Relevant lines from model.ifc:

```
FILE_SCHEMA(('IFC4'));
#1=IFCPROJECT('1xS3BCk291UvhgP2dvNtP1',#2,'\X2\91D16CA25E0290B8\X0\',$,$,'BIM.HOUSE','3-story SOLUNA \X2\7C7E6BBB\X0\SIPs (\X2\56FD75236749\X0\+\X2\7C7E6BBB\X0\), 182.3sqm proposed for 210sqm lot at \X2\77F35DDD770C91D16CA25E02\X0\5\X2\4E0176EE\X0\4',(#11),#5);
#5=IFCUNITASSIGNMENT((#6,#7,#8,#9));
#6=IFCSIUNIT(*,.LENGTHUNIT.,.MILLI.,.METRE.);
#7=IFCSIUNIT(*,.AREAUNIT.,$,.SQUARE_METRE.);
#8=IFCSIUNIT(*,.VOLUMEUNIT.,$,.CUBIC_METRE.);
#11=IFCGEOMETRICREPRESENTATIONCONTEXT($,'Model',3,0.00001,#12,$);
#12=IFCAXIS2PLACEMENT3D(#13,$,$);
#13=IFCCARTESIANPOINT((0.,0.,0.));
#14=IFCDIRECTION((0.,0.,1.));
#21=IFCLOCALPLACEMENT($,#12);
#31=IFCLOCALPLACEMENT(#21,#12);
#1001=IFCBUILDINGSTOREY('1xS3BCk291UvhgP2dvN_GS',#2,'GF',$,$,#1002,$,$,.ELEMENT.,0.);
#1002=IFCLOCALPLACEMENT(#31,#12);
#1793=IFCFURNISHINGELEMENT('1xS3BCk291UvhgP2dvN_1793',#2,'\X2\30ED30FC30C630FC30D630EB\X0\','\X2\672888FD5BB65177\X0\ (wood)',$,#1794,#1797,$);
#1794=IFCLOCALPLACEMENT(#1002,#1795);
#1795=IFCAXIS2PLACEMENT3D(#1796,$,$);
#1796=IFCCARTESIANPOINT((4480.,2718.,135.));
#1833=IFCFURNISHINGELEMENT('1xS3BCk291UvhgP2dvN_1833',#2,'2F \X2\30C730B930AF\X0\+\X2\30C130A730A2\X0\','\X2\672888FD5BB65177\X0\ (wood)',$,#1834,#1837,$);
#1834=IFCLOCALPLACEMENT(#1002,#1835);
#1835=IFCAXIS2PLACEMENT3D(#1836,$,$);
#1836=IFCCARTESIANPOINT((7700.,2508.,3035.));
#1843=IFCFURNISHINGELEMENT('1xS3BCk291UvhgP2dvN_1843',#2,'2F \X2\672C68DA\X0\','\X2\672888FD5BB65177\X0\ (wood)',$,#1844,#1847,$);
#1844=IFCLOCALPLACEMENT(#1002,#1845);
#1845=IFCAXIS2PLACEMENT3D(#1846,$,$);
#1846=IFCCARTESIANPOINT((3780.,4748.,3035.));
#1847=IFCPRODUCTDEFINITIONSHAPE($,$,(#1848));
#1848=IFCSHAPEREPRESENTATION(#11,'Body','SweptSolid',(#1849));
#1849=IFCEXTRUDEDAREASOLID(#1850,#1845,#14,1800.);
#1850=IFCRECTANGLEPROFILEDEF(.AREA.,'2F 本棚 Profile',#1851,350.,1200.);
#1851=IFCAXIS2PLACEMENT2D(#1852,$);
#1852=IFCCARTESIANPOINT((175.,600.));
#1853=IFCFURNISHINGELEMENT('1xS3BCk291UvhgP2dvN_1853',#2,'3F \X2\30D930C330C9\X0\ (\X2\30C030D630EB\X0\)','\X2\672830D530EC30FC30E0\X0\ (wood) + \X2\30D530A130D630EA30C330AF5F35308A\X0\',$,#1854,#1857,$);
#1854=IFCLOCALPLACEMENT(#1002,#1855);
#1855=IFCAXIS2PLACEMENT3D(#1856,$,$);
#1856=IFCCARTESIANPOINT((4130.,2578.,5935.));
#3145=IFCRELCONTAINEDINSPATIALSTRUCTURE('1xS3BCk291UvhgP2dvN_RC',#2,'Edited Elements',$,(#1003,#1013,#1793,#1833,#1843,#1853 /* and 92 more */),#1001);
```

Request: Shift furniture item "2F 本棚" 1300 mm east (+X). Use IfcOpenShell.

```python
import ifcopenshell
import ifcopenshell.api.geometry
import ifcopenshell.util.placement
import ifcopenshell.util.unit

model = ifcopenshell.open("model.ifc")
unit_scale = ifcopenshell.util.unit.calculate_unit_scale(model)

item = model.by_guid("1xS3BCk291UvhgP2dvN_1843")
matrix = ifcopenshell.util.placement.get_local_placement(item.ObjectPlacement)
matrix[0, 3] += 1.3 / unit_scale
ifcopenshell.api.geometry.edit_object_placement(model, product=item, matrix=matrix, is_si=False)

print(ifcopenshell.util.placement.get_local_placement(item.ObjectPlacement).round(3) + 0.0)

model.write("model_edited.ifc")
```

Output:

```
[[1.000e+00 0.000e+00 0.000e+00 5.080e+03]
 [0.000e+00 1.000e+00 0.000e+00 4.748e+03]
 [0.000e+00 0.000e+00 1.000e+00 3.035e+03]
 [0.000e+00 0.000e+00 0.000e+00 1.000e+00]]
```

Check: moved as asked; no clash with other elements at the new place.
